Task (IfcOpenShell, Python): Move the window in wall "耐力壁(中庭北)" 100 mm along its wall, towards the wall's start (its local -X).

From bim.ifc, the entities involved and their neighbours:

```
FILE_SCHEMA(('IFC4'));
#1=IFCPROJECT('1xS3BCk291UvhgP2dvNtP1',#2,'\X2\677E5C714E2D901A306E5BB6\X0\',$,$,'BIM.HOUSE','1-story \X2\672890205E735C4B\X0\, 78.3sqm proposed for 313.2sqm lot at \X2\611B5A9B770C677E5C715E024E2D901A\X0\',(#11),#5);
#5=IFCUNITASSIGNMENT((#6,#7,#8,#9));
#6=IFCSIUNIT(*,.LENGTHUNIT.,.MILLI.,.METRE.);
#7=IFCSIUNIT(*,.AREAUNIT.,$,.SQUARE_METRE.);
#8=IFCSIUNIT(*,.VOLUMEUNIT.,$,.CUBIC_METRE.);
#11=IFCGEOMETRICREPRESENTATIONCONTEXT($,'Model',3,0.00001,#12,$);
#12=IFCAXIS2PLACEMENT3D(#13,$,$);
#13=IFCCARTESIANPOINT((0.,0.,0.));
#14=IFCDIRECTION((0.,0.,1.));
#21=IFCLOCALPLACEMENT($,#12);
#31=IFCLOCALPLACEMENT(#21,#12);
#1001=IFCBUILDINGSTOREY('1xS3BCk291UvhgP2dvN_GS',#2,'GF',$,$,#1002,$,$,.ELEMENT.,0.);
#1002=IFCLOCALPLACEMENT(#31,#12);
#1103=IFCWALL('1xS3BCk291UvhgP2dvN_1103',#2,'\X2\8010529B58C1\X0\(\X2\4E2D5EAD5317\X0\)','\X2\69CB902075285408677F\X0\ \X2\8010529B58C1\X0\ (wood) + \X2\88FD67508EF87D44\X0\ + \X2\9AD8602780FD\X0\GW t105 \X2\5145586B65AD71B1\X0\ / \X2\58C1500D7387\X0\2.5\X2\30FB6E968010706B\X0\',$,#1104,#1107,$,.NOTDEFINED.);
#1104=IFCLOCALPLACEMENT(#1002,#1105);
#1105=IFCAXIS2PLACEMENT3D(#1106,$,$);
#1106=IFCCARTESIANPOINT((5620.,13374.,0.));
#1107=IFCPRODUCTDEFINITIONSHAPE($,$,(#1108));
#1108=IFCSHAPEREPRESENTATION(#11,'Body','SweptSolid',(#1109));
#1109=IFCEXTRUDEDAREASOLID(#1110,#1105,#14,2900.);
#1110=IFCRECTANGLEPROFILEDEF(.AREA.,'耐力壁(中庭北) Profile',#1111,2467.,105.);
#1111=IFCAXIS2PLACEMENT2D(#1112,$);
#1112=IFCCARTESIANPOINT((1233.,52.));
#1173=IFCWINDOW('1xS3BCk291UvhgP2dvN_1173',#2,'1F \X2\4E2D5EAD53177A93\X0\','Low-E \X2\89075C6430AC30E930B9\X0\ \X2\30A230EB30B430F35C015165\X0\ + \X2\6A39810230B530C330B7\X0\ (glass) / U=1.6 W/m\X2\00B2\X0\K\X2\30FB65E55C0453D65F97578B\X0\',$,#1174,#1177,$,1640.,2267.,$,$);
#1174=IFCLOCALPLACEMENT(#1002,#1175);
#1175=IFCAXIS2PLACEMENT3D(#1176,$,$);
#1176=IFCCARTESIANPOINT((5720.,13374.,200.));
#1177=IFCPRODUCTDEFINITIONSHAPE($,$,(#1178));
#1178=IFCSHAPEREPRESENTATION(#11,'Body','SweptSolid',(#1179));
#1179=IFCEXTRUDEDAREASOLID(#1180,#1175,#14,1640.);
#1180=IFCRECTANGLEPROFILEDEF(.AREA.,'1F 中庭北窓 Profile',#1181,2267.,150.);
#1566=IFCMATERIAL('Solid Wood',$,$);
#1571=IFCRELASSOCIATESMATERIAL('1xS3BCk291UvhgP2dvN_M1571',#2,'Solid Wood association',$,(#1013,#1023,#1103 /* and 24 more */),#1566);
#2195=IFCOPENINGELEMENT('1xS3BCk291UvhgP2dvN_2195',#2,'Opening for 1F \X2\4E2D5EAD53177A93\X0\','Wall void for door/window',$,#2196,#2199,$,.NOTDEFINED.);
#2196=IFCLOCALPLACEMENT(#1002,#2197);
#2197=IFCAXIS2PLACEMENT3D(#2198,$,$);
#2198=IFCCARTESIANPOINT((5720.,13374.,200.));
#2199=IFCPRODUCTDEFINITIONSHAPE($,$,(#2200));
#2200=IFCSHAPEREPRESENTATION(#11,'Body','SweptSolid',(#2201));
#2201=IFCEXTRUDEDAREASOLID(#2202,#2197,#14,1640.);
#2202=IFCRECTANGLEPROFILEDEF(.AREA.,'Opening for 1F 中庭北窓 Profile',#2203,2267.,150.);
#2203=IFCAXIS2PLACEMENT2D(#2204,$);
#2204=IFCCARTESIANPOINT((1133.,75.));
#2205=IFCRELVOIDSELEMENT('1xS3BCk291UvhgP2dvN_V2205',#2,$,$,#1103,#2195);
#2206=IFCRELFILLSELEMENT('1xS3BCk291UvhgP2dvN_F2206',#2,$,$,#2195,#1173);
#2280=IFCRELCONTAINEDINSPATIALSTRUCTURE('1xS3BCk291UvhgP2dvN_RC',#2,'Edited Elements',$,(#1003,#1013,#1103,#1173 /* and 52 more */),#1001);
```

```python
import ifcopenshell
import ifcopenshell.api.geometry
import ifcopenshell.util.placement

model = ifcopenshell.open("bim.ifc")

window = model.by_id(1173)
opening = window.FillsVoids[0].RelatingOpeningElement
wall = opening.VoidsElements[0].RelatingBuildingElement

wall_matrix = ifcopenshell.util.placement.get_local_placement(wall.ObjectPlacement)
shift = wall_matrix[:3, 0] * -100.0
before = ifcopenshell.util.placement.get_local_placement(window.ObjectPlacement)[:3, 3].copy()

# The window is not placed relative to its opening, so move both.
for product in (opening, window):
    matrix = ifcopenshell.util.placement.get_local_placement(product.ObjectPlacement)
    matrix[:3, 3] += shift
    ifcopenshell.api.geometry.edit_object_placement(model, product=product, matrix=matrix, is_si=False)

after = ifcopenshell.util.placement.get_local_placement(window.ObjectPlacement)[:3, 3]
print("window moved by", (after - before).round(3) + 0.0)

model.write("bim_rev.ifc")
```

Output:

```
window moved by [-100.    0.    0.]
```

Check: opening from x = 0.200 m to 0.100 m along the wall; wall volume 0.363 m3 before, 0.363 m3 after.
